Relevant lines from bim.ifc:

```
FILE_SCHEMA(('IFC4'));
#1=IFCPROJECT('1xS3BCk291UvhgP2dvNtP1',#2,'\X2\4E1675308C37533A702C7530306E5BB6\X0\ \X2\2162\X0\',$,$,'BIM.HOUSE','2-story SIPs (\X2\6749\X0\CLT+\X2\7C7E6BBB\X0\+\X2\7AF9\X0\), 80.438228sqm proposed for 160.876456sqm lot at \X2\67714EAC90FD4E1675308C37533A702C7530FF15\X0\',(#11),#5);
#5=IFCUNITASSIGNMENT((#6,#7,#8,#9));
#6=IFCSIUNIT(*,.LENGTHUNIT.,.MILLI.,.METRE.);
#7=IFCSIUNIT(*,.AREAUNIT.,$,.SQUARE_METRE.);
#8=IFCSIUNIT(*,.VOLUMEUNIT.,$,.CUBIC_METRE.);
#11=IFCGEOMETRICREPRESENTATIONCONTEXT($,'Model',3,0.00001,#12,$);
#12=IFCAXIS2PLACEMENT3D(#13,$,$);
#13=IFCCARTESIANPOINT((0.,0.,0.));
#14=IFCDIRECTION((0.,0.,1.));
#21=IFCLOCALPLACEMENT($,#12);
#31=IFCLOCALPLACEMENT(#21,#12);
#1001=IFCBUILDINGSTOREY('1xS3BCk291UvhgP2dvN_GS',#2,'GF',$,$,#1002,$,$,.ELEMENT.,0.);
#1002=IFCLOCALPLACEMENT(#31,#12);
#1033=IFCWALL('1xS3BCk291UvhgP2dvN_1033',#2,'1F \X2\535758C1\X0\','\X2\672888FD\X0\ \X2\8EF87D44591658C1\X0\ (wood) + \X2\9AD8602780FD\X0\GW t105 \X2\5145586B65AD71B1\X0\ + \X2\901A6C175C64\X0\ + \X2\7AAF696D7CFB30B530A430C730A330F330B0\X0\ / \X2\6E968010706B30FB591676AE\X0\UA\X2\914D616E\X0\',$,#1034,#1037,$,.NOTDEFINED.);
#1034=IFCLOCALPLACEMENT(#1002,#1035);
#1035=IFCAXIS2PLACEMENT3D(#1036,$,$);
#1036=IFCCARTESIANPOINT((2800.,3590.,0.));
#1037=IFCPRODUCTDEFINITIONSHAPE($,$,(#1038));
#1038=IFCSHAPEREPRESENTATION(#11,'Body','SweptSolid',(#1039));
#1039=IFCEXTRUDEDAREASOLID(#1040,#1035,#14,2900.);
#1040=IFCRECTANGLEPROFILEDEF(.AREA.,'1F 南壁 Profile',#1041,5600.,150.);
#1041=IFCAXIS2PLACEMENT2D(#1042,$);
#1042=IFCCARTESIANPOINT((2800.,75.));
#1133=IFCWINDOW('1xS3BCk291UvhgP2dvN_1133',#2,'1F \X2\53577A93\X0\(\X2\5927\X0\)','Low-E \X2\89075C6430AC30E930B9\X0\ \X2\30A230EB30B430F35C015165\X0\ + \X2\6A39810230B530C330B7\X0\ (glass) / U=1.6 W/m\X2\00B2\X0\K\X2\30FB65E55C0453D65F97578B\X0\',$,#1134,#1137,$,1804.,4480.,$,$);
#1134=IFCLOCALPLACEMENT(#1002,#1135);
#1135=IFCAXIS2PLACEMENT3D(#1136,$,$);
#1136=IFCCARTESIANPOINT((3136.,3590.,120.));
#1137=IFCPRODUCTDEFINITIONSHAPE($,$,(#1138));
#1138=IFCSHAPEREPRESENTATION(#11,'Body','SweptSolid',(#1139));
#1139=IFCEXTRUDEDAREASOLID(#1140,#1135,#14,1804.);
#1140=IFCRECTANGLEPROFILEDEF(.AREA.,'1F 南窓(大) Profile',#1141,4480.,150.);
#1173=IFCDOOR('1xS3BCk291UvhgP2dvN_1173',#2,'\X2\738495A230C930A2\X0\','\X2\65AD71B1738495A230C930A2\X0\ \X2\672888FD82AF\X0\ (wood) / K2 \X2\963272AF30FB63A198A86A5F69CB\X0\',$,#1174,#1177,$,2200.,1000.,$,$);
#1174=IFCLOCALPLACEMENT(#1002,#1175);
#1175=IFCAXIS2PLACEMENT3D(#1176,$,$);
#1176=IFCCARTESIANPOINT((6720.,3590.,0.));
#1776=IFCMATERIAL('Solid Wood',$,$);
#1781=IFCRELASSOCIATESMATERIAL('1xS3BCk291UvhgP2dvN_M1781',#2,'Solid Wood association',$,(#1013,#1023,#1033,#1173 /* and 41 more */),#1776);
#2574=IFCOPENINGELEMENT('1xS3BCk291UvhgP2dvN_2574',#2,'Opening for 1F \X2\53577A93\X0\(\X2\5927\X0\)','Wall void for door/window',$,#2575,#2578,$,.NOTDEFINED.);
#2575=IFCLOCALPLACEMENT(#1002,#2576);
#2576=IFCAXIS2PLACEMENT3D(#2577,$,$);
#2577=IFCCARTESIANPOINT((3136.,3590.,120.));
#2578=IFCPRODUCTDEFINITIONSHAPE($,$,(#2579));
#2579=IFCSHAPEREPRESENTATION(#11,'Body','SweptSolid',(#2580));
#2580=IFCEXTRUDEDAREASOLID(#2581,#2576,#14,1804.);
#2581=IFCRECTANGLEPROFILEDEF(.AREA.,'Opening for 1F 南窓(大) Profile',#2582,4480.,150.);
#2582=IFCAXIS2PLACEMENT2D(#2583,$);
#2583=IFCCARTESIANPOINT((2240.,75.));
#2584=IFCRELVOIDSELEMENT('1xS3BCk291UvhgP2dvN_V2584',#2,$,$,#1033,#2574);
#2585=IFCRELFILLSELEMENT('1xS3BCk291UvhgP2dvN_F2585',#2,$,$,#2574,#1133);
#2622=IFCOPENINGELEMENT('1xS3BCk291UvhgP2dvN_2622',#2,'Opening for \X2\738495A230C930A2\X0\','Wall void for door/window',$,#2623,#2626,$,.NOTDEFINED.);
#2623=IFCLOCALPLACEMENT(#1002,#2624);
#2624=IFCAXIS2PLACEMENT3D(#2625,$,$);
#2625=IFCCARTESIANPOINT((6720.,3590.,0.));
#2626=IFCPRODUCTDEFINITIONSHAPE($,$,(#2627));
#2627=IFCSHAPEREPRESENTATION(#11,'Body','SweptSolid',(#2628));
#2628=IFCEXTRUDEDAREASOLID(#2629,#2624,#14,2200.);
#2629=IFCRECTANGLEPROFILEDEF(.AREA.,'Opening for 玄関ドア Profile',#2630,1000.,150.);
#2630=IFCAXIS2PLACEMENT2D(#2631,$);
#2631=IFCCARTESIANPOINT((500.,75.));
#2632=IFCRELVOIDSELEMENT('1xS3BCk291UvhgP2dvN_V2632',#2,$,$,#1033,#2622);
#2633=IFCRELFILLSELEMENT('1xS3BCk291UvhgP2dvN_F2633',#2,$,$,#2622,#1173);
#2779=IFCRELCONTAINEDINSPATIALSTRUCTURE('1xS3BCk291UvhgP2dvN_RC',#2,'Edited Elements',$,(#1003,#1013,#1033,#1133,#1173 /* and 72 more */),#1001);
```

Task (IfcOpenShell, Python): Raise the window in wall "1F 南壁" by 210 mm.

```python
import numpy as np
import ifcopenshell
import ifcopenshell.api.geometry
import ifcopenshell.util.placement
import ifcopenshell.util.unit

model = ifcopenshell.open("bim.ifc")
unit_scale = ifcopenshell.util.unit.calculate_unit_scale(model)

window = model.by_guid("1xS3BCk291UvhgP2dvN_1133")
opening = window.FillsVoids[0].RelatingOpeningElement
dz = 0.21 / unit_scale

shift = np.array([0.0, 0.0, dz])
# The window is not placed relative to its opening, so move both.
for product in (opening, window):
    matrix = ifcopenshell.util.placement.get_local_placement(product.ObjectPlacement)
    matrix[:3, 3] += shift
    ifcopenshell.api.geometry.edit_object_placement(model, product=product, matrix=matrix, is_si=False)

print(f"moved by {dz * unit_scale:+.3f} m")

model.write("bim_updated.ifc")
```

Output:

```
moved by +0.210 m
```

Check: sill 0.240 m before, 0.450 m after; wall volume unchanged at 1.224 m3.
